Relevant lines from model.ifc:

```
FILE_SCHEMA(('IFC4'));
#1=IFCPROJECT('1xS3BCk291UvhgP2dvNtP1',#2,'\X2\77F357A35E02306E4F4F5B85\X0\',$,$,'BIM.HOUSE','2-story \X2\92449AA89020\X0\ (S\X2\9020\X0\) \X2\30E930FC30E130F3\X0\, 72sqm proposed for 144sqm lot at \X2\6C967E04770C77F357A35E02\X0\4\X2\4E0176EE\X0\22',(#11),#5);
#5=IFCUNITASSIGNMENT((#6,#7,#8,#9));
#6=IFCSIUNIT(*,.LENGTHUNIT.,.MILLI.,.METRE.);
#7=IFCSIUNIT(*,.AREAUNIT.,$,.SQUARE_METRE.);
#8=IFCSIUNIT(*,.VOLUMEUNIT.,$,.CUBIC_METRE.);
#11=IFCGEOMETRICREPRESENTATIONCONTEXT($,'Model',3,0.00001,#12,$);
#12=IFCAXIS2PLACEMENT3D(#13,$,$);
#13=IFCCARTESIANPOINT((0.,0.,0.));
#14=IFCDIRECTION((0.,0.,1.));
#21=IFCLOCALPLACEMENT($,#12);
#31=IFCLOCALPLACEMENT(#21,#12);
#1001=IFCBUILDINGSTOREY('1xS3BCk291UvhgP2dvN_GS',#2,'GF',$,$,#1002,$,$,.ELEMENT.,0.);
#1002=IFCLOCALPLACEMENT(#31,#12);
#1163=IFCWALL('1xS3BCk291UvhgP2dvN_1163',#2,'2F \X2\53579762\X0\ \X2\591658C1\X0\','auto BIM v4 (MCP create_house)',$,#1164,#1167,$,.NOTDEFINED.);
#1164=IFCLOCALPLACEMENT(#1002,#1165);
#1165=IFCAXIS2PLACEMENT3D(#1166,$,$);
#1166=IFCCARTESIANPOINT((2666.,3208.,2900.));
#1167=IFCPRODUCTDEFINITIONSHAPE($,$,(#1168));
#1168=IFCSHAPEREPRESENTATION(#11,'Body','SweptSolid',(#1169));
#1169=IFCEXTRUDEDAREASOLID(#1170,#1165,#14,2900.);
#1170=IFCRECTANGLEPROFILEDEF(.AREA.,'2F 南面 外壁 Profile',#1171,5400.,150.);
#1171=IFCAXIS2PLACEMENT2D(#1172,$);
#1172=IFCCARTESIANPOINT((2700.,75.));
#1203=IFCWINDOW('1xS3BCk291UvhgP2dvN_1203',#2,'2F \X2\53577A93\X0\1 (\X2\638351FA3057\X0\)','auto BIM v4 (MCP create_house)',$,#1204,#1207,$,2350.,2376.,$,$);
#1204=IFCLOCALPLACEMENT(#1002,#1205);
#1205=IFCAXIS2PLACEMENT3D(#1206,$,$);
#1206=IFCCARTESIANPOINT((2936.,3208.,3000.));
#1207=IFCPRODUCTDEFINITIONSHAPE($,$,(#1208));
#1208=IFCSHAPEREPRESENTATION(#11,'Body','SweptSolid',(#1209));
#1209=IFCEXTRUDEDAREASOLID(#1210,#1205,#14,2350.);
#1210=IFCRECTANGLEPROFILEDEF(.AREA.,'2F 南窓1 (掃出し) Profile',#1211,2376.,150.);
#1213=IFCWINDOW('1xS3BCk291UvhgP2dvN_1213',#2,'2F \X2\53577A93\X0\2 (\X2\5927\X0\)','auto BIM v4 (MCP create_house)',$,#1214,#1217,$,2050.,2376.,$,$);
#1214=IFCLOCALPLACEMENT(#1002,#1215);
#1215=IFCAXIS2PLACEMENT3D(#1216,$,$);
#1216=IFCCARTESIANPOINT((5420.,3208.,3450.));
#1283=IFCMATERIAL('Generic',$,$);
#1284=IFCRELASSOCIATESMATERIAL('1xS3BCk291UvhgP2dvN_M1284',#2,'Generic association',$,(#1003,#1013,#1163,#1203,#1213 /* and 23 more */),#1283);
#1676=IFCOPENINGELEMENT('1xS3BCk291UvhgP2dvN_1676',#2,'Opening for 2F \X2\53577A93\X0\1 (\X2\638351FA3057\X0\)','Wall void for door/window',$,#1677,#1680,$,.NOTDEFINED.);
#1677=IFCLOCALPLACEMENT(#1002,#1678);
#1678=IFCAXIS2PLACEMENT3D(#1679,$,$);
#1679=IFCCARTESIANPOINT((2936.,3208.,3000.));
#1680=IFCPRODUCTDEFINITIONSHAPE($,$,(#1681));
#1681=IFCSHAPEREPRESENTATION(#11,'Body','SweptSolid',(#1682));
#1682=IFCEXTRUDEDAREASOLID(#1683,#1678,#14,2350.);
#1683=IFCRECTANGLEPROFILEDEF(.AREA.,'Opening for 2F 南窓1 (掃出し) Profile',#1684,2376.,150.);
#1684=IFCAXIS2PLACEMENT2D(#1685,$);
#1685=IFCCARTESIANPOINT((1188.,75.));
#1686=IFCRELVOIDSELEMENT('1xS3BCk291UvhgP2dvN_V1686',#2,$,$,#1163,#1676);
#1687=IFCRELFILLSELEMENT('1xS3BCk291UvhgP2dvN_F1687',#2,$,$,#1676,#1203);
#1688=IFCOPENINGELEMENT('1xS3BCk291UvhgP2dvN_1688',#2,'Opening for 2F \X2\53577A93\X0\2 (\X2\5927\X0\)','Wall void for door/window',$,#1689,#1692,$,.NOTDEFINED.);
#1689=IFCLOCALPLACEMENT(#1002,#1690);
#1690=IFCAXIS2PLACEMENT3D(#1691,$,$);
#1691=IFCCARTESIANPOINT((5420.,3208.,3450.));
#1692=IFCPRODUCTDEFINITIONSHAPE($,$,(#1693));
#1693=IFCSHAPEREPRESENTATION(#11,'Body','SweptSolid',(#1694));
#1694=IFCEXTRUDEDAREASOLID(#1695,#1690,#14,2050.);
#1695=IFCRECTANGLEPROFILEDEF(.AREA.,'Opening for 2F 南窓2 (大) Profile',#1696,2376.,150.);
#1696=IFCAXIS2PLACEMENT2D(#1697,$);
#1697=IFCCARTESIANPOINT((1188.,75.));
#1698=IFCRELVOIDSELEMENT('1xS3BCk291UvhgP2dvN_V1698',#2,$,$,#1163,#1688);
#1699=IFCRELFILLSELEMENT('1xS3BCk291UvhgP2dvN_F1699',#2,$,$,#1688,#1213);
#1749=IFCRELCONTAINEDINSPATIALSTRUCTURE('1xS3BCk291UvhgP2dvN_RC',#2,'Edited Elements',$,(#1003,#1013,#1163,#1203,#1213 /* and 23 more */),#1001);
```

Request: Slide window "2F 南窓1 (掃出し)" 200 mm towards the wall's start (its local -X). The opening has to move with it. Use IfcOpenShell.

```python
import ifcopenshell
import ifcopenshell.api.geometry
import ifcopenshell.util.placement
import ifcopenshell.util.unit

model = ifcopenshell.open("model.ifc")
unit_scale = ifcopenshell.util.unit.calculate_unit_scale(model)

window = model.by_guid("1xS3BCk291UvhgP2dvN_1203")
opening = window.FillsVoids[0].RelatingOpeningElement
wall = opening.VoidsElements[0].RelatingBuildingElement

wall_matrix = ifcopenshell.util.placement.get_local_placement(wall.ObjectPlacement)
shift = wall_matrix[:3, 0] * -0.2 / unit_scale
before = ifcopenshell.util.placement.get_local_placement(window.ObjectPlacement)[:3, 3].copy()

# The window is not placed relative to its opening, so move both.
for product in (opening, window):
    matrix = ifcopenshell.util.placement.get_local_placement(product.ObjectPlacement)
    matrix[:3, 3] += shift
    ifcopenshell.api.geometry.edit_object_placement(model, product=product, matrix=matrix, is_si=False)

after = ifcopenshell.util.placement.get_local_placement(window.ObjectPlacement)[:3, 3]
print("window moved by", (after - before).round(3) + 0.0)

model.write("model_rev.ifc")
```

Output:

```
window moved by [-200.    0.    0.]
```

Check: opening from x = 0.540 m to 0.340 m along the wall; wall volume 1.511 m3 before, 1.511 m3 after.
